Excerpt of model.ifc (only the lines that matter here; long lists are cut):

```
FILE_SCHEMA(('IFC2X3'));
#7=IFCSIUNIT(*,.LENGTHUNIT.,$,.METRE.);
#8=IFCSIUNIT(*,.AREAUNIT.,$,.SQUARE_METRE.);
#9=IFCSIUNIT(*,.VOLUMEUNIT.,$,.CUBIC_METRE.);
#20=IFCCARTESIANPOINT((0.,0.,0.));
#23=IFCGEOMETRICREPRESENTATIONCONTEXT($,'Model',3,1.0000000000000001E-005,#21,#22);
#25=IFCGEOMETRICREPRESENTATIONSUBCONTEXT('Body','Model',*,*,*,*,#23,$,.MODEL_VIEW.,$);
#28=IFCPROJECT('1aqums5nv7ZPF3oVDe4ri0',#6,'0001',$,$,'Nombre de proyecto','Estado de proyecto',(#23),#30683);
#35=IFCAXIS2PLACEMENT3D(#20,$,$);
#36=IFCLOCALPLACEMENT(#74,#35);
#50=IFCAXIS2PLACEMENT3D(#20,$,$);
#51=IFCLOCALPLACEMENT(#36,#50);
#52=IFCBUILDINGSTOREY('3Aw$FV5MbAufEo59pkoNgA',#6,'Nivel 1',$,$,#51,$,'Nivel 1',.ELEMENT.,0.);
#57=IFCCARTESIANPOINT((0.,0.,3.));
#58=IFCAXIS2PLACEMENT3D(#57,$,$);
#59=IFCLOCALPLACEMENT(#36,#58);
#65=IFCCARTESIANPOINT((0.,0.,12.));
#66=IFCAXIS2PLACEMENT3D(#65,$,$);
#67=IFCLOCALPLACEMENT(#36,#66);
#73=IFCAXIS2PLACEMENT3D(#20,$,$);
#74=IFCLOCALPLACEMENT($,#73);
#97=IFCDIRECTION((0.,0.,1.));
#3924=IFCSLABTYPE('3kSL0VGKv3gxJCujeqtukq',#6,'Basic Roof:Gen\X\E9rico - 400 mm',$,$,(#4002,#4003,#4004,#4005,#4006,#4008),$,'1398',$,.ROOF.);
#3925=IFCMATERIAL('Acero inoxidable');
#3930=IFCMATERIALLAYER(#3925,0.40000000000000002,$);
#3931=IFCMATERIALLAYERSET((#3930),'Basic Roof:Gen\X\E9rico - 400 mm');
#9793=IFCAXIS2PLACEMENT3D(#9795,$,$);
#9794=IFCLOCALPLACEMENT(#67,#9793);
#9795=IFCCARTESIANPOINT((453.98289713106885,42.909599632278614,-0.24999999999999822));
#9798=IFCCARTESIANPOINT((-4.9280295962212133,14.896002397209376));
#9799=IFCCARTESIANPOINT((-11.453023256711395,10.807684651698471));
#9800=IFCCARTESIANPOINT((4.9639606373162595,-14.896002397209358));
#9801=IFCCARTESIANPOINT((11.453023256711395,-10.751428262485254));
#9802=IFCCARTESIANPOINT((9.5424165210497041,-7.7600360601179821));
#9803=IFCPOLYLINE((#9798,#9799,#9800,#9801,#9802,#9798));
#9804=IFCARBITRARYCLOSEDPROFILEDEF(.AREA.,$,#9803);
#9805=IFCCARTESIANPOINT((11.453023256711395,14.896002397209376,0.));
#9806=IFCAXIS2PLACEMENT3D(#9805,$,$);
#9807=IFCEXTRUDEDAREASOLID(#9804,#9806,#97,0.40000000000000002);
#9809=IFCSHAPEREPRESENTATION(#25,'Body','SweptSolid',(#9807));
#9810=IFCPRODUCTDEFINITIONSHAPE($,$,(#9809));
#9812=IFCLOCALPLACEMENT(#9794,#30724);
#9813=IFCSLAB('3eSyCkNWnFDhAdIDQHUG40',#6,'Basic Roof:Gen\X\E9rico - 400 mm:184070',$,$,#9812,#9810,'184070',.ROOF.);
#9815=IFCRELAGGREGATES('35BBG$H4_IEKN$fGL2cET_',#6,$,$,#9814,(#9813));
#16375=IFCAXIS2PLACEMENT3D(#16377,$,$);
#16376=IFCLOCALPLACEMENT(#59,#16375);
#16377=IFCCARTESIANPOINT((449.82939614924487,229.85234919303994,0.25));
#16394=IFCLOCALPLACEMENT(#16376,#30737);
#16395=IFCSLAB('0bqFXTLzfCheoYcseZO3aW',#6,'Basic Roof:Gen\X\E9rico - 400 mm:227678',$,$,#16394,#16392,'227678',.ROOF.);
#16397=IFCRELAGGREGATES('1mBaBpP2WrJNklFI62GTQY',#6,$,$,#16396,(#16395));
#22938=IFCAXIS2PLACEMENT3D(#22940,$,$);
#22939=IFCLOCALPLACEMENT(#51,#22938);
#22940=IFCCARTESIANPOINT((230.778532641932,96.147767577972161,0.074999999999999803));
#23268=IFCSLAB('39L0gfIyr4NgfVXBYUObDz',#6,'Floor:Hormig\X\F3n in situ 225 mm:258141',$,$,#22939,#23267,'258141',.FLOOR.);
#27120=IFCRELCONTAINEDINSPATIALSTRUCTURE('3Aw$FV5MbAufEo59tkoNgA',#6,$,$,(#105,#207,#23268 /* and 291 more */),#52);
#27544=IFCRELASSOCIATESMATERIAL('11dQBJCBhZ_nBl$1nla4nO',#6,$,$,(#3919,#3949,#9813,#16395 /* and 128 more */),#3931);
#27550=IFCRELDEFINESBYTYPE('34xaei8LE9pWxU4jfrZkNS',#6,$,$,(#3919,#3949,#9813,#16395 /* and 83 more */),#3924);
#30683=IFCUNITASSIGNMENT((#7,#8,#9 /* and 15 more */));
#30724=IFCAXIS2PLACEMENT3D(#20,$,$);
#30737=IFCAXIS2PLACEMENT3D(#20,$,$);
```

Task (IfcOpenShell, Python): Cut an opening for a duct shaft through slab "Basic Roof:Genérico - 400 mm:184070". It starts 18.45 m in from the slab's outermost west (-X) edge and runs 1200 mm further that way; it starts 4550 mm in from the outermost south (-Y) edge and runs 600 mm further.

```python
import numpy as np
import ifcopenshell
import ifcopenshell.api.feature
import ifcopenshell.api.geometry
import ifcopenshell.api.root
import ifcopenshell.geom
import ifcopenshell.util.placement
import ifcopenshell.util.representation
import ifcopenshell.util.shape
import ifcopenshell.util.unit

model = ifcopenshell.open("model.ifc")
unit_scale = ifcopenshell.util.unit.calculate_unit_scale(model)
settings = ifcopenshell.geom.settings()


def volume(element):
    """Net volume in cubic metres, openings subtracted."""
    shape = ifcopenshell.geom.create_shape(settings, element)
    return ifcopenshell.util.shape.get_volume(shape.geometry)


slab = model.by_id(9813)
before = volume(slab)

# Extent in the slab's own axes, in metres. The edges named are its -X and -Y sides.
slab_shape = ifcopenshell.geom.create_shape(settings, slab)
vertices = ifcopenshell.util.shape.get_vertices(slab_shape.geometry)
x_min, y_min, bottom = vertices.min(axis=0)
top = vertices[:, 2].max()

opening = ifcopenshell.api.root.create_entity(model, ifc_class="IfcOpeningElement", name="Duct shaft opening")
context = ifcopenshell.util.representation.get_context(model, "Model", "Body", "MODEL_VIEW")
width, depth = 1.2, 0.6
outline = [(0.0, 0.0), (width, 0.0), (width, depth), (0.0, depth), (0.0, 0.0)]
# Overshoot both faces by 50 mm so the cut is clean.
shape = ifcopenshell.api.geometry.add_slab_representation(
    model, context=context, depth=top - bottom + 0.1, polyline=outline
)
ifcopenshell.api.geometry.assign_representation(model, product=opening, representation=shape)

matrix = ifcopenshell.util.placement.get_local_placement(slab.ObjectPlacement)
matrix[:, 3] = matrix @ np.append(np.array([x_min + 18.45, y_min + 4.55, bottom - 0.05]) / unit_scale, 1.0)
ifcopenshell.api.geometry.edit_object_placement(model, product=opening, matrix=matrix, is_si=False)
ifcopenshell.api.feature.add_feature(model, feature=opening, element=slab)

after = volume(slab)

print(f"slab volume {before:.3f} -> {after:.3f} m3")

model.write("model_rev.ifc")
```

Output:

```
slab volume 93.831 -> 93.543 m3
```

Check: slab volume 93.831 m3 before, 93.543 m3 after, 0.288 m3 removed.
